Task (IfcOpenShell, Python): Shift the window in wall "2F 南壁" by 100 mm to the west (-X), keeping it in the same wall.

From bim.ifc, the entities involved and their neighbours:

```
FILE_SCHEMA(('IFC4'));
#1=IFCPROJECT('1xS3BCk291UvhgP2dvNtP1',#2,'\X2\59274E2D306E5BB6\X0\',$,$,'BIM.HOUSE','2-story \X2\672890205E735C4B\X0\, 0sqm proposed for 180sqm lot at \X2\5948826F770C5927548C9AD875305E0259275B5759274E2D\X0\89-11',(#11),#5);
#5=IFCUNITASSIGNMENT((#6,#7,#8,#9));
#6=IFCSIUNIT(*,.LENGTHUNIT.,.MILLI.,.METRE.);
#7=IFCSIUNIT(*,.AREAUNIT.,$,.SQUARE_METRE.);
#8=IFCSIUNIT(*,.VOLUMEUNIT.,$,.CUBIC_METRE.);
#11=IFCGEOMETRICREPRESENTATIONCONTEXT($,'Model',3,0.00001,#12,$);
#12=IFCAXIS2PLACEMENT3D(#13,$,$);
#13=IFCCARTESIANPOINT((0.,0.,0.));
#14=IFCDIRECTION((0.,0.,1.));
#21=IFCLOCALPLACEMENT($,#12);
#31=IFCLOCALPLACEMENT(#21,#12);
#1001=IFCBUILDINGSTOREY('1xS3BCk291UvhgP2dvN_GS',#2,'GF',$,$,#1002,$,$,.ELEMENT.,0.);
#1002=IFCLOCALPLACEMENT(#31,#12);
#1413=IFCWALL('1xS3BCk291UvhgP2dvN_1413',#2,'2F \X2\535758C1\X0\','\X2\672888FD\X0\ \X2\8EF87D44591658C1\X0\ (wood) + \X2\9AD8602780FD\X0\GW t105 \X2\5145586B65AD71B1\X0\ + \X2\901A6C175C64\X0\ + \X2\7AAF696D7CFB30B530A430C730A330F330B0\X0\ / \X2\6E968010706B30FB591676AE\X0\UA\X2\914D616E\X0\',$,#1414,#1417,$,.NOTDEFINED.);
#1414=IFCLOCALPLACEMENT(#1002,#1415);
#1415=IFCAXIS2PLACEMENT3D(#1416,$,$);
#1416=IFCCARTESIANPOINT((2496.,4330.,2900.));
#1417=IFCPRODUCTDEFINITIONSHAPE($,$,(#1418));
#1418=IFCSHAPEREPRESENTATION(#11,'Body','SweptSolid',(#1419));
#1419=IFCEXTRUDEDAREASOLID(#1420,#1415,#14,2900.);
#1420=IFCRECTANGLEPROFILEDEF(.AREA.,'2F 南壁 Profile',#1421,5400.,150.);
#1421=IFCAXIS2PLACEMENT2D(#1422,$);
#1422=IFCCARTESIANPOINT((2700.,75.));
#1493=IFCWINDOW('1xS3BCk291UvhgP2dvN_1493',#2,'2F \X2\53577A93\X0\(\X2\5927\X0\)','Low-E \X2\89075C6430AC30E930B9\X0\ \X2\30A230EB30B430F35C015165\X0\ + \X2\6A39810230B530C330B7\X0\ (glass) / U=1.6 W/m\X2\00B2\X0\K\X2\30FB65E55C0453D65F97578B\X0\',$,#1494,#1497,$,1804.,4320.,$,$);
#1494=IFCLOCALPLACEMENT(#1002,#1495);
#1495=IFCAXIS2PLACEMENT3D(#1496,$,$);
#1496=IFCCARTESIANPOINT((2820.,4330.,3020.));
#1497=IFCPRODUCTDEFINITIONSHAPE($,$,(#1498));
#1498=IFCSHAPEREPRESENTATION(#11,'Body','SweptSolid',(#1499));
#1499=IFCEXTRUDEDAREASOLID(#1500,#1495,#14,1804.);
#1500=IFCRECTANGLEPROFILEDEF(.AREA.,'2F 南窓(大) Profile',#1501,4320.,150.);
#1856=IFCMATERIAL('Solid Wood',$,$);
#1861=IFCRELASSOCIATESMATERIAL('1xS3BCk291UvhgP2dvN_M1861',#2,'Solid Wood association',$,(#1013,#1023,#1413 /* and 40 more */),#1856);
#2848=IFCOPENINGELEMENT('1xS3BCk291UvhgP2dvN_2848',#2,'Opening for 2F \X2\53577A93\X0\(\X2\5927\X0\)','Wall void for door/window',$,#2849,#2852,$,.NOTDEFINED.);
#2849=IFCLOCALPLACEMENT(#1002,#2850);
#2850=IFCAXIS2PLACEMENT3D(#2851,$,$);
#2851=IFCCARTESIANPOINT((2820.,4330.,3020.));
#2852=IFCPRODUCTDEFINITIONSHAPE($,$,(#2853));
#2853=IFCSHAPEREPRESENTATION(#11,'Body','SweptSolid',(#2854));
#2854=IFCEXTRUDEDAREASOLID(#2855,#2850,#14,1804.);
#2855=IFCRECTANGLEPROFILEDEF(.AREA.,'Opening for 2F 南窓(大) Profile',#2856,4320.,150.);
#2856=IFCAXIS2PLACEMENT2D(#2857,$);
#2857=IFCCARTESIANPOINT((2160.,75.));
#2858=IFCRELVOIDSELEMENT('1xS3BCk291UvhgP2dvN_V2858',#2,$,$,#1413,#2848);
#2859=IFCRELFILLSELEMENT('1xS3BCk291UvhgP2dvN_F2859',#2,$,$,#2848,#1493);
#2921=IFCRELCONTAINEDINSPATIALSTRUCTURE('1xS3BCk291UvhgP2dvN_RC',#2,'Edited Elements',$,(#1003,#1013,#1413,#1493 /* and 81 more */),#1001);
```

```python
import ifcopenshell
import ifcopenshell.api.geometry
import ifcopenshell.util.placement

model = ifcopenshell.open("bim.ifc")

window = model.by_guid("1xS3BCk291UvhgP2dvN_1493")
opening = window.FillsVoids[0].RelatingOpeningElement
wall = opening.VoidsElements[0].RelatingBuildingElement

wall_matrix = ifcopenshell.util.placement.get_local_placement(wall.ObjectPlacement)
shift = wall_matrix[:3, 0] * -100.0
before = ifcopenshell.util.placement.get_local_placement(window.ObjectPlacement)[:3, 3].copy()

# The window is not placed relative to its opening, so move both.
for product in (opening, window):
    matrix = ifcopenshell.util.placement.get_local_placement(product.ObjectPlacement)
    matrix[:3, 3] += shift
    ifcopenshell.api.geometry.edit_object_placement(model, product=product, matrix=matrix, is_si=False)

after = ifcopenshell.util.placement.get_local_placement(window.ObjectPlacement)[:3, 3]
print("window moved by", (after - before).round(3) + 0.0)

model.write("bim_updated.ifc")
```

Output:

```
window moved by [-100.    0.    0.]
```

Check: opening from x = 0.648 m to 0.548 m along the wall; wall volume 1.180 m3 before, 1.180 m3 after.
